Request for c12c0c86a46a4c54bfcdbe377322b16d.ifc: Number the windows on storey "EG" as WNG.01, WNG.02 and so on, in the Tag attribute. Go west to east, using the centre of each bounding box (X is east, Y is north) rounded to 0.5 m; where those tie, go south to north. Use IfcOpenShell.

First a look at what the model holds.

```python
import ifcopenshell
import ifcopenshell.util.element
import ifcopenshell.util.placement

model = ifcopenshell.open("c12c0c86a46a4c54bfcdbe377322b16d.ifc")
print(model.schema)
storey = next(s for s in model.by_type("IfcBuildingStorey") if s.Name == "EG")
windows = [e for e in ifcopenshell.util.element.get_decomposition(storey) if e.is_a("IfcWindow")]
for e in sorted(windows, key=lambda e: e.id()):
    origin = ifcopenshell.util.placement.get_local_placement(e.ObjectPlacement)[:3, 3]
    print(e.id(), e.Tag, e.Name, origin.round(2) + 0.0, sep=" | ")
```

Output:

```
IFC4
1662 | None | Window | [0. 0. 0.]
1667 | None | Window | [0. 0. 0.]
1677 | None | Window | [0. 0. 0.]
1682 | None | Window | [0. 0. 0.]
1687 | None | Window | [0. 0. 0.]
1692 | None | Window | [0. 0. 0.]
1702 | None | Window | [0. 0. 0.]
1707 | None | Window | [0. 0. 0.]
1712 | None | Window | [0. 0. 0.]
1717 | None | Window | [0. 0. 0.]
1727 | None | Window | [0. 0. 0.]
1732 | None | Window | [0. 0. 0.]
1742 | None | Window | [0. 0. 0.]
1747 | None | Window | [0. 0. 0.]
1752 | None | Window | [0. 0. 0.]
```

```python
import ifcopenshell
import ifcopenshell.geom
import ifcopenshell.util.element
import ifcopenshell.util.shape

model = ifcopenshell.open("c12c0c86a46a4c54bfcdbe377322b16d.ifc")
settings = ifcopenshell.geom.settings()
settings.set("use-world-coords", True)


def centre(element):
    shape = ifcopenshell.geom.create_shape(settings, element)
    return ifcopenshell.util.shape.get_bbox_centroid(shape.geometry)


storey = next(s for s in model.by_type("IfcBuildingStorey") if s.Name == "EG")
windows = [e for e in ifcopenshell.util.element.get_decomposition(storey) if e.is_a("IfcWindow")]

# Insertion points can sit at a corner or the storey origin, so sort by the geometry (in metres).
centres = {e: centre(e) for e in windows}
windows.sort(key=lambda e: (round(centres[e][0] / 0.5), centres[e][1]))

for i, e in enumerate(windows, start=1):
    number = f"WNG.{i:02d}"
    e.Tag = number
    print(e.id(), number)

model.write("c12c0c86a46a4c54bfcdbe377322b16d_updated.ifc")
```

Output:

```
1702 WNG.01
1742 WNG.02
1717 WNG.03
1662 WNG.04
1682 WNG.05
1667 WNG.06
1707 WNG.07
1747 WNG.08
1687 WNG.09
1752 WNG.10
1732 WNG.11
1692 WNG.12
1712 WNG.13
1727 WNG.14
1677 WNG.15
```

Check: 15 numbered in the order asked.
